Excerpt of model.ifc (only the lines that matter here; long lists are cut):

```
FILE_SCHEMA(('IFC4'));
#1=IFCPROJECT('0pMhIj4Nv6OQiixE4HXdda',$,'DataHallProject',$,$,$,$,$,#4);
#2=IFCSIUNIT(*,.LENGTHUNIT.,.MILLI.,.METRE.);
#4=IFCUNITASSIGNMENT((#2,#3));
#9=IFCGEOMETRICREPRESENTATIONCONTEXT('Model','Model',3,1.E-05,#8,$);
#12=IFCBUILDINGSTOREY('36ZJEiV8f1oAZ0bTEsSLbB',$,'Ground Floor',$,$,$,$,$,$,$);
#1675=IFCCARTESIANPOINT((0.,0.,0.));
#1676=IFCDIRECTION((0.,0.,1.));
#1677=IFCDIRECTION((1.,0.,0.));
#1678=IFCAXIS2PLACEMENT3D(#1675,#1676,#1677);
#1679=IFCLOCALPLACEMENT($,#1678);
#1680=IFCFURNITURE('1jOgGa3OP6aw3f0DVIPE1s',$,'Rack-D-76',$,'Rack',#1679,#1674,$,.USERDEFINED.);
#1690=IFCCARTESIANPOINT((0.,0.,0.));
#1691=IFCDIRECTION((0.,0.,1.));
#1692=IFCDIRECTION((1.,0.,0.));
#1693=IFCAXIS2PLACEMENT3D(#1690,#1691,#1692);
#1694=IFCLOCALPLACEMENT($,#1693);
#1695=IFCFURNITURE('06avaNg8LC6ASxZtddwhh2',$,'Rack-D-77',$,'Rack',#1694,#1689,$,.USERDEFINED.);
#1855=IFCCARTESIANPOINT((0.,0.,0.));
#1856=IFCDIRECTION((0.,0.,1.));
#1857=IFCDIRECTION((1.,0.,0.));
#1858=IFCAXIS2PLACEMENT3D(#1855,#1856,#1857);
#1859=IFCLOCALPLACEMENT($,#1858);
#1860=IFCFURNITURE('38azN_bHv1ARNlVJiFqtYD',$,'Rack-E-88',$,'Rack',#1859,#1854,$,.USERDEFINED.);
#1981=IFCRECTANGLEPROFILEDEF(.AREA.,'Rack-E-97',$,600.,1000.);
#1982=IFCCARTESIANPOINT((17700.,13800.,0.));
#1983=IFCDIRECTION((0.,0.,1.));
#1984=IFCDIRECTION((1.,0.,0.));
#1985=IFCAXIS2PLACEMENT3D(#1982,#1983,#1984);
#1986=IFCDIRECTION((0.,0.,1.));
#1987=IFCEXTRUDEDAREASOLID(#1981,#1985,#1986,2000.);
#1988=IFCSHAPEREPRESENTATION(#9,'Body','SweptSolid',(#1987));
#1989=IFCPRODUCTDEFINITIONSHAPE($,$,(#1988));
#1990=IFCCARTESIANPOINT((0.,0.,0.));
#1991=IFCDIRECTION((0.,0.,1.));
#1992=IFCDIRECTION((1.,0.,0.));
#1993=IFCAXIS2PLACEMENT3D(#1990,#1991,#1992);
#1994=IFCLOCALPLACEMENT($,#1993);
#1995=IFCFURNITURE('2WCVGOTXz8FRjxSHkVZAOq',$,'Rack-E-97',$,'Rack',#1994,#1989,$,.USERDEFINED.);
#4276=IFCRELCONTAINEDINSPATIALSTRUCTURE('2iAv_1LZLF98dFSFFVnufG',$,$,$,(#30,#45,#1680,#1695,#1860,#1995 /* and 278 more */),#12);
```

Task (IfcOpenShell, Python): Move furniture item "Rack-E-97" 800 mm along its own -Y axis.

```python
import ifcopenshell
import ifcopenshell.api.geometry
import ifcopenshell.util.placement
import ifcopenshell.util.unit

model = ifcopenshell.open("model.ifc")
unit_scale = ifcopenshell.util.unit.calculate_unit_scale(model)

item = model.by_guid("2WCVGOTXz8FRjxSHkVZAOq")
matrix = ifcopenshell.util.placement.get_local_placement(item.ObjectPlacement)
matrix[:3, 3] -= matrix[:3, 1] * 0.8 / unit_scale
ifcopenshell.api.geometry.edit_object_placement(model, product=item, matrix=matrix, is_si=False)

print(ifcopenshell.util.placement.get_local_placement(item.ObjectPlacement).round(3) + 0.0)

model.write("model-out.ifc")
```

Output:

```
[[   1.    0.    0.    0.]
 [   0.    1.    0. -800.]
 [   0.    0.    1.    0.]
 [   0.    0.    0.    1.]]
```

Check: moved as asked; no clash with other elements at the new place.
